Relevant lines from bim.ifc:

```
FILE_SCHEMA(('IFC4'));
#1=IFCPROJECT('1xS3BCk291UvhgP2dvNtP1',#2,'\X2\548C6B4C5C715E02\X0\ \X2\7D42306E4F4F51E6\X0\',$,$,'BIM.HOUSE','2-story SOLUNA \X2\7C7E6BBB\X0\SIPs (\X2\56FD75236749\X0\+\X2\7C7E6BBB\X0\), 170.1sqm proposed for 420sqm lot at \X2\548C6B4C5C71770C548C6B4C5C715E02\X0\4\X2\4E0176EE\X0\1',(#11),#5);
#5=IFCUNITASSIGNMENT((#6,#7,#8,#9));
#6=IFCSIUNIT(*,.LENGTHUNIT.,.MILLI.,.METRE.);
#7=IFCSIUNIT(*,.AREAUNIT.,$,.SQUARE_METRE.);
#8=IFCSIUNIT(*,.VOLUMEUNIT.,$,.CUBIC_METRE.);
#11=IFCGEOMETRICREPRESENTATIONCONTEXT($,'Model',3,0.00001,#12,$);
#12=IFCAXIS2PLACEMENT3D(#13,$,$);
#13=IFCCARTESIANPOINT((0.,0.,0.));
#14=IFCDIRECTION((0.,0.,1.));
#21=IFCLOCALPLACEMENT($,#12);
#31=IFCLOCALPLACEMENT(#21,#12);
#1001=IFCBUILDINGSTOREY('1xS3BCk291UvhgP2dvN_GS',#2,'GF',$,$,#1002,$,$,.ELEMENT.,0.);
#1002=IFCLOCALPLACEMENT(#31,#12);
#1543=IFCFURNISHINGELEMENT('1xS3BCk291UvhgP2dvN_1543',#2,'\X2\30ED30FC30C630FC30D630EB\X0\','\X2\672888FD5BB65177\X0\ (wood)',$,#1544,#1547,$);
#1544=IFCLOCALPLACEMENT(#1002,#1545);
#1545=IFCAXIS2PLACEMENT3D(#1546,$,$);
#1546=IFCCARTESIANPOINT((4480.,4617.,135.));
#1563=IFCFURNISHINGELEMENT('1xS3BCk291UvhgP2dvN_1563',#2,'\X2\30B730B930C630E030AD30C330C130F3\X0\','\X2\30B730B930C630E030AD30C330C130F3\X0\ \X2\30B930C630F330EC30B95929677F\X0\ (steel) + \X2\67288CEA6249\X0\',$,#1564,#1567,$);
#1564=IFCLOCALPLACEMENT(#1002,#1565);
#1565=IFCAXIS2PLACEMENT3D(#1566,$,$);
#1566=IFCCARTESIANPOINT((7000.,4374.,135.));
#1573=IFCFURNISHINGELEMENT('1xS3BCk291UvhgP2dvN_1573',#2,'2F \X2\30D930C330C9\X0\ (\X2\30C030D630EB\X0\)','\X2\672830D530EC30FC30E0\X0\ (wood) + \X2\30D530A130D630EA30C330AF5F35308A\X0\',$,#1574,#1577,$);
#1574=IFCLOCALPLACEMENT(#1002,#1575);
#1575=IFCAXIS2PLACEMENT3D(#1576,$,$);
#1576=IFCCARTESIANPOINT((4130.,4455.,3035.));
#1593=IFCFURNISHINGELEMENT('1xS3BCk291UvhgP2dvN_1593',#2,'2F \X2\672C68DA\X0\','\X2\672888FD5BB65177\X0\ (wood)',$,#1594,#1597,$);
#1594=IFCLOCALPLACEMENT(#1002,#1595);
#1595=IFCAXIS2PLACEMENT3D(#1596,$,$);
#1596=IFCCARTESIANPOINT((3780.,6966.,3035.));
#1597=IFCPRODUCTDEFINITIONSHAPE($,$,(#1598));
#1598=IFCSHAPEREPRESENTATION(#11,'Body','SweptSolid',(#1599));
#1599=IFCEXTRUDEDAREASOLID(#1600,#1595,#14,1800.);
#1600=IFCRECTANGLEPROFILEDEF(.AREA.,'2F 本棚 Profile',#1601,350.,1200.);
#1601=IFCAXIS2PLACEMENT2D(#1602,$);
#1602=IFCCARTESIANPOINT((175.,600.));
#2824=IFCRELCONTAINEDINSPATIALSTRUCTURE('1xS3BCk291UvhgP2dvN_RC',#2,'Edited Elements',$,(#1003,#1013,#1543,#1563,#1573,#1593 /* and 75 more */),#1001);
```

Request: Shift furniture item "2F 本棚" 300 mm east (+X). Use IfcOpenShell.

```python
import ifcopenshell
import ifcopenshell.api.geometry
import ifcopenshell.util.placement
import ifcopenshell.util.unit

model = ifcopenshell.open("bim.ifc")
unit_scale = ifcopenshell.util.unit.calculate_unit_scale(model)

item = model.by_guid("1xS3BCk291UvhgP2dvN_1593")
matrix = ifcopenshell.util.placement.get_local_placement(item.ObjectPlacement)
matrix[0, 3] += 0.3 / unit_scale
ifcopenshell.api.geometry.edit_object_placement(model, product=item, matrix=matrix, is_si=False)

print(ifcopenshell.util.placement.get_local_placement(item.ObjectPlacement).round(3) + 0.0)

model.write("bim_rev.ifc")
```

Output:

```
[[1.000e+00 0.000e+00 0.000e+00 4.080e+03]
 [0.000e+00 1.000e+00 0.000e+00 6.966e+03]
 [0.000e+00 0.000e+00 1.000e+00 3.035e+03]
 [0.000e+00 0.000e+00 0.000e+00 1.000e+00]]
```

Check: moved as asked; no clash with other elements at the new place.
